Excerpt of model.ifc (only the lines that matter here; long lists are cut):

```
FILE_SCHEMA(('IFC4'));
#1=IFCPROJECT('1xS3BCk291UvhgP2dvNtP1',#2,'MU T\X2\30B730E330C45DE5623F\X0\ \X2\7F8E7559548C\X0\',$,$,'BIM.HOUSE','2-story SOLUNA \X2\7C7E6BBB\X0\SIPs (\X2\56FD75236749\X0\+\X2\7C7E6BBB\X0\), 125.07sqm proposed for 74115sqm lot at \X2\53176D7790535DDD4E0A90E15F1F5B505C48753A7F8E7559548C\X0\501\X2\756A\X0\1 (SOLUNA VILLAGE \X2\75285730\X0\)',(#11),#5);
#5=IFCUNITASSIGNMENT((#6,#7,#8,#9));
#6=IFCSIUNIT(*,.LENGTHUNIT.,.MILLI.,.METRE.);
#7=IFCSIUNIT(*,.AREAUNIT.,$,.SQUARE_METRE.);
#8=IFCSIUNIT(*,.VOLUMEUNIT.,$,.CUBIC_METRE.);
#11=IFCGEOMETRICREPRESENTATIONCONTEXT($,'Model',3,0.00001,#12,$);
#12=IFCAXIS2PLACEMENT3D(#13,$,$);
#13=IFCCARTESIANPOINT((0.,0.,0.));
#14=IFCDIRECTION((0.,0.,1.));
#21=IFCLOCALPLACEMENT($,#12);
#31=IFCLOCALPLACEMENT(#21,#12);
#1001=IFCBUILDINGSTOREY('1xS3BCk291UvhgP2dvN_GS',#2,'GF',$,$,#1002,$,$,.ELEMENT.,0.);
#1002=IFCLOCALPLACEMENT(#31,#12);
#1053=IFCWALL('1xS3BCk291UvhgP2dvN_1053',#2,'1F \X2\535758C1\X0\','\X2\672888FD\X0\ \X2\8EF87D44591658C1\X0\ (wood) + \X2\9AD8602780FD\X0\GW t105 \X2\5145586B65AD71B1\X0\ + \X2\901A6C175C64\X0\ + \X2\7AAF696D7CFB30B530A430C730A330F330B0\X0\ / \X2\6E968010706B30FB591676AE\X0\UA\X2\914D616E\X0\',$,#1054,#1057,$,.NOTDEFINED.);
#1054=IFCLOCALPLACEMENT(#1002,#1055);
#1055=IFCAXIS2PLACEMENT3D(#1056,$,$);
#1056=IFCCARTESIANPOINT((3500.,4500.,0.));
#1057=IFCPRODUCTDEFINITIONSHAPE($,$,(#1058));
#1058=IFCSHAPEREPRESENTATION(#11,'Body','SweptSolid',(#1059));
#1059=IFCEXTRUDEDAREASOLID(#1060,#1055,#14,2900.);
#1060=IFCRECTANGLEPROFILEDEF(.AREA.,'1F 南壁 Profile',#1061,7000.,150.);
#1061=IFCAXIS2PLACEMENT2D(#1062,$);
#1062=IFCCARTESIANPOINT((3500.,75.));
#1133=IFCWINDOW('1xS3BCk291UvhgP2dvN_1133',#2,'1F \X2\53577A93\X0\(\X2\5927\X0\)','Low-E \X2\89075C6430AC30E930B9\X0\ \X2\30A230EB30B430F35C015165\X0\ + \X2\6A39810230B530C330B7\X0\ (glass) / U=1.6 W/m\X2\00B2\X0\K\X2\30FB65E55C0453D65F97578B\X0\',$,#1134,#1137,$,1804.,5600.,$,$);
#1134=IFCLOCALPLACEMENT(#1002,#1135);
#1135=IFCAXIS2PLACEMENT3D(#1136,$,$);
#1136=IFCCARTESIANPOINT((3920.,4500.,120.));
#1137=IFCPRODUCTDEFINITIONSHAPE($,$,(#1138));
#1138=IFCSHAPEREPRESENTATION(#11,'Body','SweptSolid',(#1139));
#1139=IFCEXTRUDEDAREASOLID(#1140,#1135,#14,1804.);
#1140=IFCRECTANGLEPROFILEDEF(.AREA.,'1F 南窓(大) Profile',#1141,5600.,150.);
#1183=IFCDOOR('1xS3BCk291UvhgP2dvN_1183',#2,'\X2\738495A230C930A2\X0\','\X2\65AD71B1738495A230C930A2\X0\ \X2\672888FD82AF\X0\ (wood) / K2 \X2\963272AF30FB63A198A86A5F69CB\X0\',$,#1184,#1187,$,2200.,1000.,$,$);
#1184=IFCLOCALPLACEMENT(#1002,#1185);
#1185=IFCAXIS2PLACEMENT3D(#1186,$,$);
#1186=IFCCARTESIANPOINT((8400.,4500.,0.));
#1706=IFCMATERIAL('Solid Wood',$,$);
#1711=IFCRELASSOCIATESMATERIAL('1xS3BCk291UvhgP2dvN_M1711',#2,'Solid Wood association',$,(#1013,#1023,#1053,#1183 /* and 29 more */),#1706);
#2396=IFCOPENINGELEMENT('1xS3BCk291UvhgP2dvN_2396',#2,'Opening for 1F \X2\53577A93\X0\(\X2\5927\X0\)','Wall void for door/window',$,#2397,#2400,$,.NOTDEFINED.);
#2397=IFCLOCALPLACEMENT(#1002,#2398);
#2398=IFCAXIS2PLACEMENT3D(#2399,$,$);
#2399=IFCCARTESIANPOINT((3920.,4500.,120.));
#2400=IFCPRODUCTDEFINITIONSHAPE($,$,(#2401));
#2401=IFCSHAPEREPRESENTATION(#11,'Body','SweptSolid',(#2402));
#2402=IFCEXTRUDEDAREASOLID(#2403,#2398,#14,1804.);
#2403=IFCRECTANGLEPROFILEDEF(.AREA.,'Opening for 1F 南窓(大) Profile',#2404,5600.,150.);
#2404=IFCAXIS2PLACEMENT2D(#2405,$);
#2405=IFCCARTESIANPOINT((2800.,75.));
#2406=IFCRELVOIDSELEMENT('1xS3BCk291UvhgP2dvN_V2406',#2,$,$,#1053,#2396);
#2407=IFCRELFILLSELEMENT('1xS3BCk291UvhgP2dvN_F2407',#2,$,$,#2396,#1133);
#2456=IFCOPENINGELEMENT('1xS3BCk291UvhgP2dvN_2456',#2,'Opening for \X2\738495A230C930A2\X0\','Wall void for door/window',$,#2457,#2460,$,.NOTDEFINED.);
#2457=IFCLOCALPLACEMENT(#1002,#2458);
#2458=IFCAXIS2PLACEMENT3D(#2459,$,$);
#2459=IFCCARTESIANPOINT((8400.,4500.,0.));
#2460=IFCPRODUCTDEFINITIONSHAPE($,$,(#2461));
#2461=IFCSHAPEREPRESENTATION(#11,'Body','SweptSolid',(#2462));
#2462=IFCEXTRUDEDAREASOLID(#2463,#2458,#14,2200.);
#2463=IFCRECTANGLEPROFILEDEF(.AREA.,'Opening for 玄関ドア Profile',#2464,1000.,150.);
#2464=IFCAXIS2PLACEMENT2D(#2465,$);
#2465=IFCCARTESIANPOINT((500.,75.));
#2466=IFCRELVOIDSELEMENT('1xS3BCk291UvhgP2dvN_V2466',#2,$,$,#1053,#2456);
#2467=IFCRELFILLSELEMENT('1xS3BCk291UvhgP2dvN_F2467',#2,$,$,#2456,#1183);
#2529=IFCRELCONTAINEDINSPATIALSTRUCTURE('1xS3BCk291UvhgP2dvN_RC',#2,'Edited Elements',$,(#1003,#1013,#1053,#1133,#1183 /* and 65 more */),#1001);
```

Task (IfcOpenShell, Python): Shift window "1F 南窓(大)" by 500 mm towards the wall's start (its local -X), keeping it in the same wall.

```python
import ifcopenshell
import ifcopenshell.api.geometry
import ifcopenshell.util.placement

model = ifcopenshell.open("model.ifc")

window = model.by_guid("1xS3BCk291UvhgP2dvN_1133")
opening = window.FillsVoids[0].RelatingOpeningElement
wall = opening.VoidsElements[0].RelatingBuildingElement

wall_matrix = ifcopenshell.util.placement.get_local_placement(wall.ObjectPlacement)
shift = wall_matrix[:3, 0] * -500.0
before = ifcopenshell.util.placement.get_local_placement(window.ObjectPlacement)[:3, 3].copy()

# The window is not placed relative to its opening, so move both.
for product in (opening, window):
    matrix = ifcopenshell.util.placement.get_local_placement(product.ObjectPlacement)
    matrix[:3, 3] += shift
    ifcopenshell.api.geometry.edit_object_placement(model, product=product, matrix=matrix, is_si=False)

after = ifcopenshell.util.placement.get_local_placement(window.ObjectPlacement)[:3, 3]
print("window moved by", (after - before).round(3) + 0.0)

model.write("model_rev.ifc")
```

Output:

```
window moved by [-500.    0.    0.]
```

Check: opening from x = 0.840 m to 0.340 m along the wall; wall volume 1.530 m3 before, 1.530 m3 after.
